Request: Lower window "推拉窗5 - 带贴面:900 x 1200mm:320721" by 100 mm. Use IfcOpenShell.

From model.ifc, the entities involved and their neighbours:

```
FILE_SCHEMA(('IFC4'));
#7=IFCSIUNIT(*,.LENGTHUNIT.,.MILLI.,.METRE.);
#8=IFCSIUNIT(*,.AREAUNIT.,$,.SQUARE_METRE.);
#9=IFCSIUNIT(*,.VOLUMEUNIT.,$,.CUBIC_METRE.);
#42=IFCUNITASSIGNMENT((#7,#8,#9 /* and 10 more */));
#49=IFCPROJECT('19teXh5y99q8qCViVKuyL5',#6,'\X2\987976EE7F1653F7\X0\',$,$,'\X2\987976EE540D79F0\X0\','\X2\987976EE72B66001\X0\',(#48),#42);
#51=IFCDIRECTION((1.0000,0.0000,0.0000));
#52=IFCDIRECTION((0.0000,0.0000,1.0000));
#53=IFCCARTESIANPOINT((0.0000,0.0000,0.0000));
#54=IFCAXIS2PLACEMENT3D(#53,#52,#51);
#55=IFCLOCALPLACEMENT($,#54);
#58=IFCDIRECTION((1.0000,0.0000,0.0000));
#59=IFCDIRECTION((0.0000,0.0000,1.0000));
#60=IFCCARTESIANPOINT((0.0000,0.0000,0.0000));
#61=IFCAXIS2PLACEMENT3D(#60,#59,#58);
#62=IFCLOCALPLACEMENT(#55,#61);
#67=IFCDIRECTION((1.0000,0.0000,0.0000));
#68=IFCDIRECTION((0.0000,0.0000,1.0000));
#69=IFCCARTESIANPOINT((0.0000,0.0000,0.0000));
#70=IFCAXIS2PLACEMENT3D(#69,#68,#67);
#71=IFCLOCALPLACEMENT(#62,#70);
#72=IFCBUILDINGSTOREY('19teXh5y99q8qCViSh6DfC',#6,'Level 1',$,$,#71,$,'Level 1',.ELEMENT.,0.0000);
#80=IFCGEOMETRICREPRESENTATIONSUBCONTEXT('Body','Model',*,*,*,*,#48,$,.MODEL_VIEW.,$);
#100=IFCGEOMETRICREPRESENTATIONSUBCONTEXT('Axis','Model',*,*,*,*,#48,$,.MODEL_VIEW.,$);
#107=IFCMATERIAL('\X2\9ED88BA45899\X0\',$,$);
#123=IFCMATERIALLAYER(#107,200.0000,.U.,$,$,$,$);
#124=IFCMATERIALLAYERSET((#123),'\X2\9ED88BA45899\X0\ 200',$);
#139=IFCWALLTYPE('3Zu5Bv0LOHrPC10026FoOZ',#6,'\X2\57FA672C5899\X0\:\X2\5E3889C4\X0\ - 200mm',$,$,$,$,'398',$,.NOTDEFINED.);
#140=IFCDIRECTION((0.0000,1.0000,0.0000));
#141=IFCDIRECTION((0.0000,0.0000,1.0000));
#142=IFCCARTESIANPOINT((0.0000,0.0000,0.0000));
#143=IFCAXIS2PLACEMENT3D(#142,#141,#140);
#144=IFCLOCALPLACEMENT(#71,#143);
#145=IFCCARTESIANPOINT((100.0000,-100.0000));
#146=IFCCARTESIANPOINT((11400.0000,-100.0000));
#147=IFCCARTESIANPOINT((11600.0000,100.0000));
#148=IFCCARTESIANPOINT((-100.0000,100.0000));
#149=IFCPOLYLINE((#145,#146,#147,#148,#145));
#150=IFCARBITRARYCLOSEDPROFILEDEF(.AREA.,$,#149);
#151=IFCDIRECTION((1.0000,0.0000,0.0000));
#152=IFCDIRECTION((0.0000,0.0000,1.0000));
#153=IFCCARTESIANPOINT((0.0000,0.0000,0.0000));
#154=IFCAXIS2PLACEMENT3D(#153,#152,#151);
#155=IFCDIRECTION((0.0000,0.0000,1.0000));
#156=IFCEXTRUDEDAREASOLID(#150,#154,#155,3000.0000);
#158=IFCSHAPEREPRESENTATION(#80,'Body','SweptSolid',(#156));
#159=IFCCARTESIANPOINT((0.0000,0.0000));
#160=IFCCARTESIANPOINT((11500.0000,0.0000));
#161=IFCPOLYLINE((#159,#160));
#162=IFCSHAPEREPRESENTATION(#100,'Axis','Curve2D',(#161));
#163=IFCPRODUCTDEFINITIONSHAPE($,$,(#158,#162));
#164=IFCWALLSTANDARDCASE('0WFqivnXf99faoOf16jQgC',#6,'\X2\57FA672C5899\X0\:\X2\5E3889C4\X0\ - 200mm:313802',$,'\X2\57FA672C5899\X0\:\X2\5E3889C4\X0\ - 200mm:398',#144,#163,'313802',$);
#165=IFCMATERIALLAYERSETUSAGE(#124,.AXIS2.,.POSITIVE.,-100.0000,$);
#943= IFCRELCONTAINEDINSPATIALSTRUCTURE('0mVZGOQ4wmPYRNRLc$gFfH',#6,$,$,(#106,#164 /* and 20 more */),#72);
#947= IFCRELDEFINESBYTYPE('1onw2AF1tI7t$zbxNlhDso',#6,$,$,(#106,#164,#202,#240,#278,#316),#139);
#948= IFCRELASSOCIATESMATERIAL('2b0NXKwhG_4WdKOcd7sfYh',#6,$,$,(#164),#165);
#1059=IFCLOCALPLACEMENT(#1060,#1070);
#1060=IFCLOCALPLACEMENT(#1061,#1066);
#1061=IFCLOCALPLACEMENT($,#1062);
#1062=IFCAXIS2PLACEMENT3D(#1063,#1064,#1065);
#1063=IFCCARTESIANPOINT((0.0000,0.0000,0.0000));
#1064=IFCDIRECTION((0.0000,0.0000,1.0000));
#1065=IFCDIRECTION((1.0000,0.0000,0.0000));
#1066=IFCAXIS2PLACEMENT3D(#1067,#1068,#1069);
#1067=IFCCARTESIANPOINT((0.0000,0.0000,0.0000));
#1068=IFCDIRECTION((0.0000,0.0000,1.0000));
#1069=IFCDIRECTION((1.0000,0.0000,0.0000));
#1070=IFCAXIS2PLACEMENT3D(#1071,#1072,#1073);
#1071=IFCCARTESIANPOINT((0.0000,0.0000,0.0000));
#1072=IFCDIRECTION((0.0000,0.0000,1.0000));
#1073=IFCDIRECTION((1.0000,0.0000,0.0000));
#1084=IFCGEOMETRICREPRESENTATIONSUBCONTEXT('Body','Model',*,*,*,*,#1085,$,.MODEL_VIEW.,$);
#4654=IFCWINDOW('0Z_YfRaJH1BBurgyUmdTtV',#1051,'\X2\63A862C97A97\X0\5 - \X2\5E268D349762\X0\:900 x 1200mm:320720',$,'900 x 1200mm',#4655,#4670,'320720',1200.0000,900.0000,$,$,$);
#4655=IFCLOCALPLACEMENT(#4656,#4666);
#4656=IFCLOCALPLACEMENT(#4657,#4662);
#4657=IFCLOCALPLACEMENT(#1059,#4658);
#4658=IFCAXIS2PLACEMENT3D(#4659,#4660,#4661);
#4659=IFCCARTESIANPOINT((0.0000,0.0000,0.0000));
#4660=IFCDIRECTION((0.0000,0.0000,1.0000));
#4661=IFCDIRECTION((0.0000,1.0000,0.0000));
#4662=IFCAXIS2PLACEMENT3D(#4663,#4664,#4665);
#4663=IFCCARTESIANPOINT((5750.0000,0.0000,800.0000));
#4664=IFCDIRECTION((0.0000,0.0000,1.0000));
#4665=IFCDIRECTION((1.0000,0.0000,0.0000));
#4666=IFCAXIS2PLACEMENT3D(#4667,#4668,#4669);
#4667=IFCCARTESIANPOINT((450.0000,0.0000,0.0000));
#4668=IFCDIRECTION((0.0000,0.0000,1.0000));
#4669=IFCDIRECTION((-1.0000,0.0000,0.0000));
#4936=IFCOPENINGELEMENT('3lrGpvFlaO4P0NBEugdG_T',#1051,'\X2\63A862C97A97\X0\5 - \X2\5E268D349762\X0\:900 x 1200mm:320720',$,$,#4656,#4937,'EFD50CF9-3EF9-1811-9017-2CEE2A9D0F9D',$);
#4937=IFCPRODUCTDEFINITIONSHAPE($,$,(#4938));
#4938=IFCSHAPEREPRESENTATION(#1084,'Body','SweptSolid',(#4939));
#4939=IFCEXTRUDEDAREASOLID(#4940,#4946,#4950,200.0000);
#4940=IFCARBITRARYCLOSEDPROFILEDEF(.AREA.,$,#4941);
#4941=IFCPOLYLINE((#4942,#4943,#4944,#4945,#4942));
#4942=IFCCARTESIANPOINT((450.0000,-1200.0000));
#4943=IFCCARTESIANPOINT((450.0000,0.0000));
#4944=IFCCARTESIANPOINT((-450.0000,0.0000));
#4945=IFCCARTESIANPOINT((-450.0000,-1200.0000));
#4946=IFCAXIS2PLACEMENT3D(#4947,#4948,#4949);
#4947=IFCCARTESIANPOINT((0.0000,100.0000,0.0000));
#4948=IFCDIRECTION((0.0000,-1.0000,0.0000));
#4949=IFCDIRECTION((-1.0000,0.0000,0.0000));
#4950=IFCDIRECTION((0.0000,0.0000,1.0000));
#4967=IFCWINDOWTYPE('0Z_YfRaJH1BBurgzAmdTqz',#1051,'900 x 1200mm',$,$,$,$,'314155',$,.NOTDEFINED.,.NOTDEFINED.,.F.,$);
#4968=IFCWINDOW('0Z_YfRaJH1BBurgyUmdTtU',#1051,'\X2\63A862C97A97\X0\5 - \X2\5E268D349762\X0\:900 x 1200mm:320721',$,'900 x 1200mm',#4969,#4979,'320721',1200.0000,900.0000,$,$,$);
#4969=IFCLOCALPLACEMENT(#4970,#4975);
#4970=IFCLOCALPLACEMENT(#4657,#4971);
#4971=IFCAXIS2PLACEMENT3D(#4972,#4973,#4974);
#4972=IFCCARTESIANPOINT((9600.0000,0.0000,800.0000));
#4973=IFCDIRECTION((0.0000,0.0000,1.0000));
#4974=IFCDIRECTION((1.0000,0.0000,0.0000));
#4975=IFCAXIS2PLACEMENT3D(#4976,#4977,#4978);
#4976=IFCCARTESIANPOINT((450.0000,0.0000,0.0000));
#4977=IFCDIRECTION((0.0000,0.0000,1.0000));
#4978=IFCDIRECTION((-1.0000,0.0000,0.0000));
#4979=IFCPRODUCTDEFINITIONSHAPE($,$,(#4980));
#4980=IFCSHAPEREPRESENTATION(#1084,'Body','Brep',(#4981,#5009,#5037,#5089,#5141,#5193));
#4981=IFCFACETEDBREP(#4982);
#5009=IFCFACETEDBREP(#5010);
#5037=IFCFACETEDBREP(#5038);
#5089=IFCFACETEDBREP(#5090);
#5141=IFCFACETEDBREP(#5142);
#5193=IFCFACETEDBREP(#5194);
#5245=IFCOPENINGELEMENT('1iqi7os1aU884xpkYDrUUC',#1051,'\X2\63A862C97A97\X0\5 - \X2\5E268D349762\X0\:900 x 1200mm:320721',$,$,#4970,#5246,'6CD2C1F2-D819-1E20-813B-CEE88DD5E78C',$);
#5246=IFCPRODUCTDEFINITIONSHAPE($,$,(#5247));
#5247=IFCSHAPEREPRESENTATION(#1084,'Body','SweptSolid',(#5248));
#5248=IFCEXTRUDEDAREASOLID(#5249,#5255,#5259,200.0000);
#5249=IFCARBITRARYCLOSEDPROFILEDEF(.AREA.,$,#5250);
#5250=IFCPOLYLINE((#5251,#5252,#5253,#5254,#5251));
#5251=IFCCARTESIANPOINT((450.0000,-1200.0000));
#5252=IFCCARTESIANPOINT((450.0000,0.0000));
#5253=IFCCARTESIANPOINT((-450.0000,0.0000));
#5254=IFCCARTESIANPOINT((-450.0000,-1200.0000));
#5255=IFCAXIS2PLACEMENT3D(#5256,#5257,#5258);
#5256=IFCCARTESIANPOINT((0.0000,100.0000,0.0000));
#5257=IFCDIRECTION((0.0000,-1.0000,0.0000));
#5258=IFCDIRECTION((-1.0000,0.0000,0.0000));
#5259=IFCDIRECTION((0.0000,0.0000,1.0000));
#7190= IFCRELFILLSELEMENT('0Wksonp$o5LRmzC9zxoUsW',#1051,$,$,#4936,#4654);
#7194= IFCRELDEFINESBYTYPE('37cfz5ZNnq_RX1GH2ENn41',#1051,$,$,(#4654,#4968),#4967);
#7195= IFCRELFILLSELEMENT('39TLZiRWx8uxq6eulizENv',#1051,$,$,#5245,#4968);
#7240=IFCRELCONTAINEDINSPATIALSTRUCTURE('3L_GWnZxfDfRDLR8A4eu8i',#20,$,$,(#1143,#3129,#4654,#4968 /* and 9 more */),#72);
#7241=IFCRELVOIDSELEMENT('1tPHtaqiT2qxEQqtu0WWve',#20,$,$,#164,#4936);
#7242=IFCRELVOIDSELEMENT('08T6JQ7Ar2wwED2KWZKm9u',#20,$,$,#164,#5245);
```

```python
import numpy as np
import ifcopenshell
import ifcopenshell.api.geometry
import ifcopenshell.util.placement
import ifcopenshell.util.unit

model = ifcopenshell.open("model.ifc")
unit_scale = ifcopenshell.util.unit.calculate_unit_scale(model)

window = model.by_guid("0Z_YfRaJH1BBurgyUmdTtU")
opening = window.FillsVoids[0].RelatingOpeningElement
dz = -0.1 / unit_scale

shift = np.array([0.0, 0.0, dz])
# The window is placed relative to its opening, so it follows when the opening moves.
matrix = ifcopenshell.util.placement.get_local_placement(opening.ObjectPlacement)
matrix[:3, 3] += shift
ifcopenshell.api.geometry.edit_object_placement(
    model, product=opening, matrix=matrix, is_si=False, should_transform_children=True
)

print(f"moved by {dz * unit_scale:+.3f} m")

model.write("model_updated.ifc")
```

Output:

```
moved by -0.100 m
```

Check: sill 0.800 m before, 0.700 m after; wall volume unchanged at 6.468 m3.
